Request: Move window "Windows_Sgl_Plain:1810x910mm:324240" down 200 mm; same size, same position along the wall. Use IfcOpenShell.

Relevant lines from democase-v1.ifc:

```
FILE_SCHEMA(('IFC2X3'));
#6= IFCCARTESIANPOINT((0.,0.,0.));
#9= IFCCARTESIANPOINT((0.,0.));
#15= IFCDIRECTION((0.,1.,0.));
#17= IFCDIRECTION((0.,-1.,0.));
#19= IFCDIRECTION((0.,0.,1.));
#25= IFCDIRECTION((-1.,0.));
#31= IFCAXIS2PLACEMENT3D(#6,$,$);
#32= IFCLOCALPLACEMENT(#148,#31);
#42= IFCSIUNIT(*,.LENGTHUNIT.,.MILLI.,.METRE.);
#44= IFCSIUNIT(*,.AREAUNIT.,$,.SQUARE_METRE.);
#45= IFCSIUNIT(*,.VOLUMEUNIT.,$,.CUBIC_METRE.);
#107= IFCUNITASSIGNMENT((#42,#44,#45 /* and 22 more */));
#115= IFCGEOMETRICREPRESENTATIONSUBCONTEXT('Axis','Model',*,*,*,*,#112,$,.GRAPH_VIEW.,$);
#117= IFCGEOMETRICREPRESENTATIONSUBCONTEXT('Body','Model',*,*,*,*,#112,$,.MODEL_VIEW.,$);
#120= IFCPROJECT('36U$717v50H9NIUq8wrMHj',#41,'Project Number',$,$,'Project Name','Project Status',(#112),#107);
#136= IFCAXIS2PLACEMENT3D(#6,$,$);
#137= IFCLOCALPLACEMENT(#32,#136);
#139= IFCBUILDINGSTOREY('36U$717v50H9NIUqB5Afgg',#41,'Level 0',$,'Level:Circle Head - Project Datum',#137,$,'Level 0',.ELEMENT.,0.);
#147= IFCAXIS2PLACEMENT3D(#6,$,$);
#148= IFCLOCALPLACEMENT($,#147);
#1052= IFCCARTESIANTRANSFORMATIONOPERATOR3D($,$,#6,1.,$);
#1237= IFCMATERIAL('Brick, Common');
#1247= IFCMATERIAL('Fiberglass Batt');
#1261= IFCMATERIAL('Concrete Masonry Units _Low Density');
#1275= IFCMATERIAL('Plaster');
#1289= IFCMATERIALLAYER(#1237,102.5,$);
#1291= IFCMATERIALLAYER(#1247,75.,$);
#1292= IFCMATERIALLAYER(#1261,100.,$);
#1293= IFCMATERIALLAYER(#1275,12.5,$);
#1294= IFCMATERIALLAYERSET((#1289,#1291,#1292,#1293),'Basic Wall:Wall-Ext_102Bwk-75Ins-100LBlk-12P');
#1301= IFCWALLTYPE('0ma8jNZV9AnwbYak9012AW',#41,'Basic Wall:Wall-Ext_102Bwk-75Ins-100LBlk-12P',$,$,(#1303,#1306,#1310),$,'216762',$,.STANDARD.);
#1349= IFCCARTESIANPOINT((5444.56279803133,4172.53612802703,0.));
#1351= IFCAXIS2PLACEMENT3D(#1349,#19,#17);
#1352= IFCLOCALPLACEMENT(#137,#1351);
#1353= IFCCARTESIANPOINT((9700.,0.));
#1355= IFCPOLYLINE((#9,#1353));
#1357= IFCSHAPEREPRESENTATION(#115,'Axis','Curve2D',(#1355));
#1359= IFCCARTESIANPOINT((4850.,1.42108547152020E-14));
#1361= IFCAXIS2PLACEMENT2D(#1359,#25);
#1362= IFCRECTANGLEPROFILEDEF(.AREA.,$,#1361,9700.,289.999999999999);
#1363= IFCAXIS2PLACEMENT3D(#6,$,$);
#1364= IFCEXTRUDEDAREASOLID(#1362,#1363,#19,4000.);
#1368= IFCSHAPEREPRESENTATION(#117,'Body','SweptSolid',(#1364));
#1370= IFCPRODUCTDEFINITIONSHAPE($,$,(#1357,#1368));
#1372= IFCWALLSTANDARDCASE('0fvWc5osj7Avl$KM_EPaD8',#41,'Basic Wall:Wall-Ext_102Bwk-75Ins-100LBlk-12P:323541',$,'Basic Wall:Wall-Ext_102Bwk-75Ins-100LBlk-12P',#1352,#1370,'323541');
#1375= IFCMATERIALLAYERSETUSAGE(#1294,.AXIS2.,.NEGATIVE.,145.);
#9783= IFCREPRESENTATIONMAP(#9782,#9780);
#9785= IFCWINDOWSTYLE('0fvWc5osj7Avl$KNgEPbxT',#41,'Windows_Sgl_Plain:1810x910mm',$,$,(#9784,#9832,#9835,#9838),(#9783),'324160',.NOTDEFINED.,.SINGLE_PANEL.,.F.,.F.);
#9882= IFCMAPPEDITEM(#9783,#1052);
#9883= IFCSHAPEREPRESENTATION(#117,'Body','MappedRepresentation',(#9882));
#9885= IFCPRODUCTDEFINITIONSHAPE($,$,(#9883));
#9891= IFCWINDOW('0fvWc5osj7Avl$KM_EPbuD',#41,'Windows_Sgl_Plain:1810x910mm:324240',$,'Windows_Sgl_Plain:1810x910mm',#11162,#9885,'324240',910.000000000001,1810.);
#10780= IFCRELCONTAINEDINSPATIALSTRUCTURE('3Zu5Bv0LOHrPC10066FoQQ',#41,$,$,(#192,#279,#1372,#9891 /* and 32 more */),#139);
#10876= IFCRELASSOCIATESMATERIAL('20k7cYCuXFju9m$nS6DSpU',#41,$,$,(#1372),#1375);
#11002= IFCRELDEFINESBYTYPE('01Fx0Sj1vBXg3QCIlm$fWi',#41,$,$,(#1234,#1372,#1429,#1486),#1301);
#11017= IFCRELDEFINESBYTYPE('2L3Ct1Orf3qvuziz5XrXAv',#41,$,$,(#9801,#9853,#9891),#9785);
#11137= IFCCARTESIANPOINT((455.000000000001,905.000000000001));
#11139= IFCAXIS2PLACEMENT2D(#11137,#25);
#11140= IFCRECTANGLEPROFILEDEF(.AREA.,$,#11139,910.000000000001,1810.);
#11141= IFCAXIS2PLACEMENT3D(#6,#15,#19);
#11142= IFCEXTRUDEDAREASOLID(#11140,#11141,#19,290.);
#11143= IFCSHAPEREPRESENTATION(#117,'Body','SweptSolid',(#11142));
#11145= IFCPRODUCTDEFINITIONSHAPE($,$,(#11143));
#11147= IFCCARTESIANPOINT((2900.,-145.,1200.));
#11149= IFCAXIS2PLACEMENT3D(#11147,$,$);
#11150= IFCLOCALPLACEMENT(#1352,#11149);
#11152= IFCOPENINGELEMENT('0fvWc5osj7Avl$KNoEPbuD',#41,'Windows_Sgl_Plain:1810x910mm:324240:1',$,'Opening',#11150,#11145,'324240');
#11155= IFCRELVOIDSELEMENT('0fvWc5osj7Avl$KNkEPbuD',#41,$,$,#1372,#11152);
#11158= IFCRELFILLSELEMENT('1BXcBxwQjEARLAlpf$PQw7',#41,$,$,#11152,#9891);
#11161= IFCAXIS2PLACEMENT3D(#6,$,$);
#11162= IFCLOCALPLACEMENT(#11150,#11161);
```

```python
import numpy as np
import ifcopenshell
import ifcopenshell.api.geometry
import ifcopenshell.util.placement
import ifcopenshell.util.unit

model = ifcopenshell.open("democase-v1.ifc")
unit_scale = ifcopenshell.util.unit.calculate_unit_scale(model)

window = model.by_id(9891)
opening = window.FillsVoids[0].RelatingOpeningElement
dz = -0.2 / unit_scale

shift = np.array([0.0, 0.0, dz])
# The window is placed relative to its opening, so it follows when the opening moves.
matrix = ifcopenshell.util.placement.get_local_placement(opening.ObjectPlacement)
matrix[:3, 3] += shift
ifcopenshell.api.geometry.edit_object_placement(
    model, product=opening, matrix=matrix, is_si=False, should_transform_children=True
)

print(f"moved by {dz * unit_scale:+.3f} m")

model.write("democase-v1_updated.ifc")
```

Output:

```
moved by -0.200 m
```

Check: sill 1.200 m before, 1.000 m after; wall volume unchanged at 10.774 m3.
